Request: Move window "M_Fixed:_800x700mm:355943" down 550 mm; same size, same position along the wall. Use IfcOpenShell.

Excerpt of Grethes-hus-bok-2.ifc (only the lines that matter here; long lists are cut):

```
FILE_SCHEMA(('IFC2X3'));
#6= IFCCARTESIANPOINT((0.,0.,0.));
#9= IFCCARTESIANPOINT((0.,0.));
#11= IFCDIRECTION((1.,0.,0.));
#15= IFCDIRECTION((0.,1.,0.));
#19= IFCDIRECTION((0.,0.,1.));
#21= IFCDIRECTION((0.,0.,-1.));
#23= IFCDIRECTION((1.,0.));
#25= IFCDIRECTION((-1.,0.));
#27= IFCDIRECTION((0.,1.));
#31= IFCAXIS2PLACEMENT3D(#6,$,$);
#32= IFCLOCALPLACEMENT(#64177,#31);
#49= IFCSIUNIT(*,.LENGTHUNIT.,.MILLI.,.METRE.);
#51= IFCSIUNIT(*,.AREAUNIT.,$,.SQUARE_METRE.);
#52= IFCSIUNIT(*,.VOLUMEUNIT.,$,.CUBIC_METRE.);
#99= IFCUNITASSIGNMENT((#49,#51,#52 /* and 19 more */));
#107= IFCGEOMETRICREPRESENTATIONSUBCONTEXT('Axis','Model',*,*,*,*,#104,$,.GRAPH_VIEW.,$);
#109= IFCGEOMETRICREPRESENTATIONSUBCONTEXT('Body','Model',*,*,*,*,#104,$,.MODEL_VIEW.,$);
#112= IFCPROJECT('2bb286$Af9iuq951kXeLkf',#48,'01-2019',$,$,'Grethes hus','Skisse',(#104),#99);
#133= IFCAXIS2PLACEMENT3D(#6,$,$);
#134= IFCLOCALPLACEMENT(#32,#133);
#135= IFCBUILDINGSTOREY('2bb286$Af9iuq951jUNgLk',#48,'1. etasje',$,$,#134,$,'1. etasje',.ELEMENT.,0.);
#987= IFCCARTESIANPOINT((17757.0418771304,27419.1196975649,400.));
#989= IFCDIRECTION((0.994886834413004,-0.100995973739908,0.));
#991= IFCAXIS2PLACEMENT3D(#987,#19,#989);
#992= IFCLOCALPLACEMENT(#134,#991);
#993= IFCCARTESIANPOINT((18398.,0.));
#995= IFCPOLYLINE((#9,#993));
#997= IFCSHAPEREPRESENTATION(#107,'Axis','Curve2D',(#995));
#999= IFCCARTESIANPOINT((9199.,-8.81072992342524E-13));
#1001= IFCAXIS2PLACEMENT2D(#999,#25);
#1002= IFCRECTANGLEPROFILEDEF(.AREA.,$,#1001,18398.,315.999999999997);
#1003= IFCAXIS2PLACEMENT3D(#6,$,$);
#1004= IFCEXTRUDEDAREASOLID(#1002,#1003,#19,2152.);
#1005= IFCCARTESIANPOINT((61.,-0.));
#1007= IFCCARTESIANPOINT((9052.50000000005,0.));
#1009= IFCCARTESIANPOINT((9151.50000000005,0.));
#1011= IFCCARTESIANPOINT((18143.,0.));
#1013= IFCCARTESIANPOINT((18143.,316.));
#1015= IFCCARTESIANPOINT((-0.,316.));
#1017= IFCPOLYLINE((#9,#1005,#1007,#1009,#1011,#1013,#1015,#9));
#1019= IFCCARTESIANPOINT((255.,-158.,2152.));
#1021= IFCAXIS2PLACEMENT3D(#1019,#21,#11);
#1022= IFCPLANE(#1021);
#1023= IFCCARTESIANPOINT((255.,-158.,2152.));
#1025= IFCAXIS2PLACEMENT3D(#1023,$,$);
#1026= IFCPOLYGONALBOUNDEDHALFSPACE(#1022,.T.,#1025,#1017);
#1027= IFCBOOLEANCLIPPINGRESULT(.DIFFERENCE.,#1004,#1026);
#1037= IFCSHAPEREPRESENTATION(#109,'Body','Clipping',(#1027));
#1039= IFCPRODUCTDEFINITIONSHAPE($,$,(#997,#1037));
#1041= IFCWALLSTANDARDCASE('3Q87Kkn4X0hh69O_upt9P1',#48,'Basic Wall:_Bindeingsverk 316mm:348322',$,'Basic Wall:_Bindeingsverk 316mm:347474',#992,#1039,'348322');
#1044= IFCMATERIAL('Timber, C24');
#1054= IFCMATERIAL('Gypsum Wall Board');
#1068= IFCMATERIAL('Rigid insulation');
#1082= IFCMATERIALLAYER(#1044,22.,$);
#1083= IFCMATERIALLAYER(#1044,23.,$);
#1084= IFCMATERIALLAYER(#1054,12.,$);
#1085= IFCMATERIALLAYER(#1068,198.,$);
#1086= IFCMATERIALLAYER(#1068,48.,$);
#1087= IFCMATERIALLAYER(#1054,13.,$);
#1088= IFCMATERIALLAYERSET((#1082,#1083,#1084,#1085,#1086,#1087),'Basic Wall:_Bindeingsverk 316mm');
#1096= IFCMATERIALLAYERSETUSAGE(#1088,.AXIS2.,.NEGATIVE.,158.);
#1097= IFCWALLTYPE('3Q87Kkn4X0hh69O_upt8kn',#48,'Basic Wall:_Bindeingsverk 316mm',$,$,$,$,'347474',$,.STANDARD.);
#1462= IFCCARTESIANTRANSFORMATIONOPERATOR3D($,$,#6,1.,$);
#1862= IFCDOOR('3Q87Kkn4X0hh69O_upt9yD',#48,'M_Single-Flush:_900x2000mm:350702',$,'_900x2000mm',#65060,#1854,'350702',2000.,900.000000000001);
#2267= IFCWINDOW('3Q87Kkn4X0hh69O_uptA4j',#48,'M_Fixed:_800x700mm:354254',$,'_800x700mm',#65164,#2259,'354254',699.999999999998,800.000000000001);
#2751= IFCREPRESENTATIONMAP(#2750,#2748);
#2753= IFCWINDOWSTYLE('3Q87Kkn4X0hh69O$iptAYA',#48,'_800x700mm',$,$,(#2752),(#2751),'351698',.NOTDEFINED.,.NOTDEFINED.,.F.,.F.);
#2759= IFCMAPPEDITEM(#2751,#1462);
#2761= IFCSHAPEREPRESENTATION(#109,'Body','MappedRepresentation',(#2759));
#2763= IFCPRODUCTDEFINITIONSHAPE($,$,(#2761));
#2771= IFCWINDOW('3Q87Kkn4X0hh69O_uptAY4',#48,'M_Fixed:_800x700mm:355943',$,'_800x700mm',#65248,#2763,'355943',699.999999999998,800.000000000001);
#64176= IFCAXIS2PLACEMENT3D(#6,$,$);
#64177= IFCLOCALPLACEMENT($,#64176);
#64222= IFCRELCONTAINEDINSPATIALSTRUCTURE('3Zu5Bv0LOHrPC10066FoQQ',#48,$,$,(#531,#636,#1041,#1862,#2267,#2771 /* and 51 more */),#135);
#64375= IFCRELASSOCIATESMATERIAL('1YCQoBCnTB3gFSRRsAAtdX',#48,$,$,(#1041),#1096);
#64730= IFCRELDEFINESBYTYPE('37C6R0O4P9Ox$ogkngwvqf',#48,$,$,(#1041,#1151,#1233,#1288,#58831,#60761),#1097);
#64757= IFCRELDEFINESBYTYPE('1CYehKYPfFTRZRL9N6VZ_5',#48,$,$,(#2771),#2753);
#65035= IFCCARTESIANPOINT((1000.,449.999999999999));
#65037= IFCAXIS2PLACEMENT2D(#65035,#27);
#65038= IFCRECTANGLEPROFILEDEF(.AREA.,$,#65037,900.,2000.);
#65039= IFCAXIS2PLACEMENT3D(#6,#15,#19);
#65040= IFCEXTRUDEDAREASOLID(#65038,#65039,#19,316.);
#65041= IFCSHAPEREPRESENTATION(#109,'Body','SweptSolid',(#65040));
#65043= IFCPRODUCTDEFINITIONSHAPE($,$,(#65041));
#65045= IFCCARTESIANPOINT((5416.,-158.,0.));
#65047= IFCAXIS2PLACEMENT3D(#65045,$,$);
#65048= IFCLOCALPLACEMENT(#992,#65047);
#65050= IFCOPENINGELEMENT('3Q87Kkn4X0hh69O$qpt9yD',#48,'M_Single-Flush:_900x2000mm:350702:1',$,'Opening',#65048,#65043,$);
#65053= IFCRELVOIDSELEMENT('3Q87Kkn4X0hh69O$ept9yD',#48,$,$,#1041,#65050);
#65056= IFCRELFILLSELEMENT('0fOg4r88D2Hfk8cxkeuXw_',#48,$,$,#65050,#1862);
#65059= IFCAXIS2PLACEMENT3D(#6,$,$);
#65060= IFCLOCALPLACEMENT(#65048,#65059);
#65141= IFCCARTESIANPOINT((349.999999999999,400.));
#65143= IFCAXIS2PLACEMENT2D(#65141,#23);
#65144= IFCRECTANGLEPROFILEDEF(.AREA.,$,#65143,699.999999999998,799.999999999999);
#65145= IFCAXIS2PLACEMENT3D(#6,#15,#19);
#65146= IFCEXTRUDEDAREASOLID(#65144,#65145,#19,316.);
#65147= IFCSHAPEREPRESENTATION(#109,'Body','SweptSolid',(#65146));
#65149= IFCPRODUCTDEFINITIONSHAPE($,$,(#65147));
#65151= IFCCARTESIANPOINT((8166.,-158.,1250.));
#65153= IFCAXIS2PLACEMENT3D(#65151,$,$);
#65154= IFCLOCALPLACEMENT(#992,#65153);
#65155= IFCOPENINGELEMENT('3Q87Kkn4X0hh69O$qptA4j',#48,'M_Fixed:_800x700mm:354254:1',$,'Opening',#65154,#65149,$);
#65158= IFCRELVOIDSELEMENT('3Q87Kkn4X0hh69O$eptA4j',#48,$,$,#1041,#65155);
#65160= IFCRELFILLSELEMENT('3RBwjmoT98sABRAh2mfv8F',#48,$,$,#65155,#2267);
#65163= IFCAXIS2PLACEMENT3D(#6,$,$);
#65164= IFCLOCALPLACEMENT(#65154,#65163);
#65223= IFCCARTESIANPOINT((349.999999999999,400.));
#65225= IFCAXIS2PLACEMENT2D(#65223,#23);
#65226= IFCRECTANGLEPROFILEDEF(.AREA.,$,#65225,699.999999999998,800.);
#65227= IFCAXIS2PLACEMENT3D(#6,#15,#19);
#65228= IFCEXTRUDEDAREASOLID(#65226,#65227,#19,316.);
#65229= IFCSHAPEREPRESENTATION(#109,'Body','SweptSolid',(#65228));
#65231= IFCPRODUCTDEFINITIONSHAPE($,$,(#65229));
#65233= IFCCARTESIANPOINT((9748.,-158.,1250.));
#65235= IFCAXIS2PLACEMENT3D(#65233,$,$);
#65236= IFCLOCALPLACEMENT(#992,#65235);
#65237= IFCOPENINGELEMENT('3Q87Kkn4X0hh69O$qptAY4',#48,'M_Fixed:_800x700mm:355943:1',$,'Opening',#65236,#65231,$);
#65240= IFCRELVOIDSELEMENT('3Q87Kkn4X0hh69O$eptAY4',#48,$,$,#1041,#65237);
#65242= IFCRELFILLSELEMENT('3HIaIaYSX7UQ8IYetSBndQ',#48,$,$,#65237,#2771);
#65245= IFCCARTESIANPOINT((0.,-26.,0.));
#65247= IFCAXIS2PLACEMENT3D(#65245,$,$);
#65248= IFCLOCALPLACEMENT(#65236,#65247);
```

```python
import numpy as np
import ifcopenshell
import ifcopenshell.api.geometry
import ifcopenshell.util.placement
import ifcopenshell.util.unit

model = ifcopenshell.open("Grethes-hus-bok-2.ifc")
unit_scale = ifcopenshell.util.unit.calculate_unit_scale(model)

window = model.by_guid("3Q87Kkn4X0hh69O_uptAY4")
opening = window.FillsVoids[0].RelatingOpeningElement
dz = -550.0

shift = np.array([0.0, 0.0, dz])
# The window is placed relative to its opening, so it follows when the opening moves.
matrix = ifcopenshell.util.placement.get_local_placement(opening.ObjectPlacement)
matrix[:3, 3] += shift
ifcopenshell.api.geometry.edit_object_placement(
    model, product=opening, matrix=matrix, is_si=False, should_transform_children=True
)

print(f"moved by {dz * unit_scale:+.3f} m")

model.write("Grethes-hus-bok-2-out.ifc")
```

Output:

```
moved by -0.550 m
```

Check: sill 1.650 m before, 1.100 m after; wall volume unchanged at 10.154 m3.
